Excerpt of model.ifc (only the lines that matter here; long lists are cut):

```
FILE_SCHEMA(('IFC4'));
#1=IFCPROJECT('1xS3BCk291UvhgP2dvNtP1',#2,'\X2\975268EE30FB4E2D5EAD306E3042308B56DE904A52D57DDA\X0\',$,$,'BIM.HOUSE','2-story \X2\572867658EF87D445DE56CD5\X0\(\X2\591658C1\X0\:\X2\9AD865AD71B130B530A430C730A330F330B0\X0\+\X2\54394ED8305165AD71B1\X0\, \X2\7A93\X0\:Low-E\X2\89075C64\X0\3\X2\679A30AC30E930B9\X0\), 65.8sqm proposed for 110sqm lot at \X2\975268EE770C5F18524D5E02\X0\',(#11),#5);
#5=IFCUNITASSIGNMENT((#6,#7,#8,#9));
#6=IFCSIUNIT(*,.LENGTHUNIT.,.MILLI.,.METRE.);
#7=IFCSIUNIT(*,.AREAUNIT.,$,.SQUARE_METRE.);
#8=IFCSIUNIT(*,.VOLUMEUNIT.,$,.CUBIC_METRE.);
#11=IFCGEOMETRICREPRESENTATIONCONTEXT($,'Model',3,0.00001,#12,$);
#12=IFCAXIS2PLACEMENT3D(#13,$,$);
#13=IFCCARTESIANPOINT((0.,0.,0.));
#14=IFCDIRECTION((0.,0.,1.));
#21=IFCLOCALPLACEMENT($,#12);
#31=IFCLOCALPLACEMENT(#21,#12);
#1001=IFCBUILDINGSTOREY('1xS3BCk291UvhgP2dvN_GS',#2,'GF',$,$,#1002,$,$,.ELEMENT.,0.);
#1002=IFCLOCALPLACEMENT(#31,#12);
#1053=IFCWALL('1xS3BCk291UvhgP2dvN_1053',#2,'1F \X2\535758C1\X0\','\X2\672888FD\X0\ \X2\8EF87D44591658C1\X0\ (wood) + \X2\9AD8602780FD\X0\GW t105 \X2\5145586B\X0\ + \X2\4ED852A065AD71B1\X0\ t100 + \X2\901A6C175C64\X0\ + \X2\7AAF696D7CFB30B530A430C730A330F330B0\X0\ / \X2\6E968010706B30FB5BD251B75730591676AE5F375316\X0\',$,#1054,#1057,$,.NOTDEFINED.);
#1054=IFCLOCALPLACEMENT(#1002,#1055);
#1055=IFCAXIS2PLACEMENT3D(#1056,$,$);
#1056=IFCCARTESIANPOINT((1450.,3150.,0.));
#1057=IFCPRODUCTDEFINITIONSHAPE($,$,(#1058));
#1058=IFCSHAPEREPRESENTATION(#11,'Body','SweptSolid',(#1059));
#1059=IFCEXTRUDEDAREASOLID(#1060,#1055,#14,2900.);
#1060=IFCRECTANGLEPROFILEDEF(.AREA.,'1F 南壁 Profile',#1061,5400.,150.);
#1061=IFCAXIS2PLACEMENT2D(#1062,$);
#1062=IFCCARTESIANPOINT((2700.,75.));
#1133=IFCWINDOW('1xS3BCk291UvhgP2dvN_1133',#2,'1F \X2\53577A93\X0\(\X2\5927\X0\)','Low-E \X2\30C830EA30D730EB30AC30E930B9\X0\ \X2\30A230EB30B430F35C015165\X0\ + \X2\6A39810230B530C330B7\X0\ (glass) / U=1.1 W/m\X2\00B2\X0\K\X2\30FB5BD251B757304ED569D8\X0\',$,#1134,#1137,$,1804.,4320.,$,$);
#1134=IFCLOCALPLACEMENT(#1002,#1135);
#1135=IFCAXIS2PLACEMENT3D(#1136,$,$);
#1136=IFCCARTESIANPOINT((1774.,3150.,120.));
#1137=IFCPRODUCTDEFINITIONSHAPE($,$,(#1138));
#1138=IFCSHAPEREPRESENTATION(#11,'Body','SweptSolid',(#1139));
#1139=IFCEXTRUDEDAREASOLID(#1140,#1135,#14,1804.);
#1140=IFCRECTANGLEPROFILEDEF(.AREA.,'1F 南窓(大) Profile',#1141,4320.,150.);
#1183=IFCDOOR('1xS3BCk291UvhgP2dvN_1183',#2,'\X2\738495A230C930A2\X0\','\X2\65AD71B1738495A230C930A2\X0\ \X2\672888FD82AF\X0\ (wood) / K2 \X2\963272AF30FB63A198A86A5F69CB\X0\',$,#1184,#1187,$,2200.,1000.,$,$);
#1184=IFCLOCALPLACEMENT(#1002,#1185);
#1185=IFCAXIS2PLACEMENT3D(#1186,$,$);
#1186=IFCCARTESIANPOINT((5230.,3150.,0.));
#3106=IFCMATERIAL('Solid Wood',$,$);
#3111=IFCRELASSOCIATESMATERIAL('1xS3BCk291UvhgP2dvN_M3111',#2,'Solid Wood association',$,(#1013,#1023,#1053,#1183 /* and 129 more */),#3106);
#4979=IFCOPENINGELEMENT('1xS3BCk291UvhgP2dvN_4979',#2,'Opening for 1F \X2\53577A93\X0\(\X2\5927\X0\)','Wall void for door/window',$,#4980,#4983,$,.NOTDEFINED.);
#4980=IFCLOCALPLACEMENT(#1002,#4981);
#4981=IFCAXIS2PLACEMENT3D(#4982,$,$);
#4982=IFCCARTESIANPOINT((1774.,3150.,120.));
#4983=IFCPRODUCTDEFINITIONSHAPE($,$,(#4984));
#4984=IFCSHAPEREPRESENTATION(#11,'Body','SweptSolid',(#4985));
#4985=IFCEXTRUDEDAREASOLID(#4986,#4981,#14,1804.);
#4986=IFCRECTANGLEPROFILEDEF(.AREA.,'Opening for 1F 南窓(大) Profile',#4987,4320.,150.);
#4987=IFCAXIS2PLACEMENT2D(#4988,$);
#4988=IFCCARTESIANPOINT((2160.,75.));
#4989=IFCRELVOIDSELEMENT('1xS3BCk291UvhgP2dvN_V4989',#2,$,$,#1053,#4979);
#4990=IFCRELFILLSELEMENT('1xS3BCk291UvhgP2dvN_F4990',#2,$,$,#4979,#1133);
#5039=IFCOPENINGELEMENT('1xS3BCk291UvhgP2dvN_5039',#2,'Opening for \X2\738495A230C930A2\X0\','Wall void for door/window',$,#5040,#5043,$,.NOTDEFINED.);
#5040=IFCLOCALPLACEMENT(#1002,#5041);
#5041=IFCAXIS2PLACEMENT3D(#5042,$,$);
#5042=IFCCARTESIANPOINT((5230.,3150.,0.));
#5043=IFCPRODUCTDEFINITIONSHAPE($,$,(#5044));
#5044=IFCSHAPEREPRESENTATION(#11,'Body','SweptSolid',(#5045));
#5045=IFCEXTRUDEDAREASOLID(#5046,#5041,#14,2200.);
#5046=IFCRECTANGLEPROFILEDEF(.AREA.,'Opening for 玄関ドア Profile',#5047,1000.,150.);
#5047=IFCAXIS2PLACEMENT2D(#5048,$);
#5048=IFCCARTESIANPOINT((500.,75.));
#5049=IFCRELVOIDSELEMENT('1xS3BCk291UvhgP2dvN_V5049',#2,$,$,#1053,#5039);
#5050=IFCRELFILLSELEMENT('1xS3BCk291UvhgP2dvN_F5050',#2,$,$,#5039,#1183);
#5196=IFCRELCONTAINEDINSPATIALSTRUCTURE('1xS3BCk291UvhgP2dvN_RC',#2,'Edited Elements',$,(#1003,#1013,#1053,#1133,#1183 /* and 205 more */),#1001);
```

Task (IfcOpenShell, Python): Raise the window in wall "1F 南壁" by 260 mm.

```python
import numpy as np
import ifcopenshell
import ifcopenshell.api.geometry
import ifcopenshell.util.placement
import ifcopenshell.util.unit

model = ifcopenshell.open("model.ifc")
unit_scale = ifcopenshell.util.unit.calculate_unit_scale(model)

window = model.by_guid("1xS3BCk291UvhgP2dvN_1133")
opening = window.FillsVoids[0].RelatingOpeningElement
dz = 0.26 / unit_scale

shift = np.array([0.0, 0.0, dz])
# The window is not placed relative to its opening, so move both.
for product in (opening, window):
    matrix = ifcopenshell.util.placement.get_local_placement(product.ObjectPlacement)
    matrix[:3, 3] += shift
    ifcopenshell.api.geometry.edit_object_placement(model, product=product, matrix=matrix, is_si=False)

print(f"moved by {dz * unit_scale:+.3f} m")

model.write("model_updated.ifc")
```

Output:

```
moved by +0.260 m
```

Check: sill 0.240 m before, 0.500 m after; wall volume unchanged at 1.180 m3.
